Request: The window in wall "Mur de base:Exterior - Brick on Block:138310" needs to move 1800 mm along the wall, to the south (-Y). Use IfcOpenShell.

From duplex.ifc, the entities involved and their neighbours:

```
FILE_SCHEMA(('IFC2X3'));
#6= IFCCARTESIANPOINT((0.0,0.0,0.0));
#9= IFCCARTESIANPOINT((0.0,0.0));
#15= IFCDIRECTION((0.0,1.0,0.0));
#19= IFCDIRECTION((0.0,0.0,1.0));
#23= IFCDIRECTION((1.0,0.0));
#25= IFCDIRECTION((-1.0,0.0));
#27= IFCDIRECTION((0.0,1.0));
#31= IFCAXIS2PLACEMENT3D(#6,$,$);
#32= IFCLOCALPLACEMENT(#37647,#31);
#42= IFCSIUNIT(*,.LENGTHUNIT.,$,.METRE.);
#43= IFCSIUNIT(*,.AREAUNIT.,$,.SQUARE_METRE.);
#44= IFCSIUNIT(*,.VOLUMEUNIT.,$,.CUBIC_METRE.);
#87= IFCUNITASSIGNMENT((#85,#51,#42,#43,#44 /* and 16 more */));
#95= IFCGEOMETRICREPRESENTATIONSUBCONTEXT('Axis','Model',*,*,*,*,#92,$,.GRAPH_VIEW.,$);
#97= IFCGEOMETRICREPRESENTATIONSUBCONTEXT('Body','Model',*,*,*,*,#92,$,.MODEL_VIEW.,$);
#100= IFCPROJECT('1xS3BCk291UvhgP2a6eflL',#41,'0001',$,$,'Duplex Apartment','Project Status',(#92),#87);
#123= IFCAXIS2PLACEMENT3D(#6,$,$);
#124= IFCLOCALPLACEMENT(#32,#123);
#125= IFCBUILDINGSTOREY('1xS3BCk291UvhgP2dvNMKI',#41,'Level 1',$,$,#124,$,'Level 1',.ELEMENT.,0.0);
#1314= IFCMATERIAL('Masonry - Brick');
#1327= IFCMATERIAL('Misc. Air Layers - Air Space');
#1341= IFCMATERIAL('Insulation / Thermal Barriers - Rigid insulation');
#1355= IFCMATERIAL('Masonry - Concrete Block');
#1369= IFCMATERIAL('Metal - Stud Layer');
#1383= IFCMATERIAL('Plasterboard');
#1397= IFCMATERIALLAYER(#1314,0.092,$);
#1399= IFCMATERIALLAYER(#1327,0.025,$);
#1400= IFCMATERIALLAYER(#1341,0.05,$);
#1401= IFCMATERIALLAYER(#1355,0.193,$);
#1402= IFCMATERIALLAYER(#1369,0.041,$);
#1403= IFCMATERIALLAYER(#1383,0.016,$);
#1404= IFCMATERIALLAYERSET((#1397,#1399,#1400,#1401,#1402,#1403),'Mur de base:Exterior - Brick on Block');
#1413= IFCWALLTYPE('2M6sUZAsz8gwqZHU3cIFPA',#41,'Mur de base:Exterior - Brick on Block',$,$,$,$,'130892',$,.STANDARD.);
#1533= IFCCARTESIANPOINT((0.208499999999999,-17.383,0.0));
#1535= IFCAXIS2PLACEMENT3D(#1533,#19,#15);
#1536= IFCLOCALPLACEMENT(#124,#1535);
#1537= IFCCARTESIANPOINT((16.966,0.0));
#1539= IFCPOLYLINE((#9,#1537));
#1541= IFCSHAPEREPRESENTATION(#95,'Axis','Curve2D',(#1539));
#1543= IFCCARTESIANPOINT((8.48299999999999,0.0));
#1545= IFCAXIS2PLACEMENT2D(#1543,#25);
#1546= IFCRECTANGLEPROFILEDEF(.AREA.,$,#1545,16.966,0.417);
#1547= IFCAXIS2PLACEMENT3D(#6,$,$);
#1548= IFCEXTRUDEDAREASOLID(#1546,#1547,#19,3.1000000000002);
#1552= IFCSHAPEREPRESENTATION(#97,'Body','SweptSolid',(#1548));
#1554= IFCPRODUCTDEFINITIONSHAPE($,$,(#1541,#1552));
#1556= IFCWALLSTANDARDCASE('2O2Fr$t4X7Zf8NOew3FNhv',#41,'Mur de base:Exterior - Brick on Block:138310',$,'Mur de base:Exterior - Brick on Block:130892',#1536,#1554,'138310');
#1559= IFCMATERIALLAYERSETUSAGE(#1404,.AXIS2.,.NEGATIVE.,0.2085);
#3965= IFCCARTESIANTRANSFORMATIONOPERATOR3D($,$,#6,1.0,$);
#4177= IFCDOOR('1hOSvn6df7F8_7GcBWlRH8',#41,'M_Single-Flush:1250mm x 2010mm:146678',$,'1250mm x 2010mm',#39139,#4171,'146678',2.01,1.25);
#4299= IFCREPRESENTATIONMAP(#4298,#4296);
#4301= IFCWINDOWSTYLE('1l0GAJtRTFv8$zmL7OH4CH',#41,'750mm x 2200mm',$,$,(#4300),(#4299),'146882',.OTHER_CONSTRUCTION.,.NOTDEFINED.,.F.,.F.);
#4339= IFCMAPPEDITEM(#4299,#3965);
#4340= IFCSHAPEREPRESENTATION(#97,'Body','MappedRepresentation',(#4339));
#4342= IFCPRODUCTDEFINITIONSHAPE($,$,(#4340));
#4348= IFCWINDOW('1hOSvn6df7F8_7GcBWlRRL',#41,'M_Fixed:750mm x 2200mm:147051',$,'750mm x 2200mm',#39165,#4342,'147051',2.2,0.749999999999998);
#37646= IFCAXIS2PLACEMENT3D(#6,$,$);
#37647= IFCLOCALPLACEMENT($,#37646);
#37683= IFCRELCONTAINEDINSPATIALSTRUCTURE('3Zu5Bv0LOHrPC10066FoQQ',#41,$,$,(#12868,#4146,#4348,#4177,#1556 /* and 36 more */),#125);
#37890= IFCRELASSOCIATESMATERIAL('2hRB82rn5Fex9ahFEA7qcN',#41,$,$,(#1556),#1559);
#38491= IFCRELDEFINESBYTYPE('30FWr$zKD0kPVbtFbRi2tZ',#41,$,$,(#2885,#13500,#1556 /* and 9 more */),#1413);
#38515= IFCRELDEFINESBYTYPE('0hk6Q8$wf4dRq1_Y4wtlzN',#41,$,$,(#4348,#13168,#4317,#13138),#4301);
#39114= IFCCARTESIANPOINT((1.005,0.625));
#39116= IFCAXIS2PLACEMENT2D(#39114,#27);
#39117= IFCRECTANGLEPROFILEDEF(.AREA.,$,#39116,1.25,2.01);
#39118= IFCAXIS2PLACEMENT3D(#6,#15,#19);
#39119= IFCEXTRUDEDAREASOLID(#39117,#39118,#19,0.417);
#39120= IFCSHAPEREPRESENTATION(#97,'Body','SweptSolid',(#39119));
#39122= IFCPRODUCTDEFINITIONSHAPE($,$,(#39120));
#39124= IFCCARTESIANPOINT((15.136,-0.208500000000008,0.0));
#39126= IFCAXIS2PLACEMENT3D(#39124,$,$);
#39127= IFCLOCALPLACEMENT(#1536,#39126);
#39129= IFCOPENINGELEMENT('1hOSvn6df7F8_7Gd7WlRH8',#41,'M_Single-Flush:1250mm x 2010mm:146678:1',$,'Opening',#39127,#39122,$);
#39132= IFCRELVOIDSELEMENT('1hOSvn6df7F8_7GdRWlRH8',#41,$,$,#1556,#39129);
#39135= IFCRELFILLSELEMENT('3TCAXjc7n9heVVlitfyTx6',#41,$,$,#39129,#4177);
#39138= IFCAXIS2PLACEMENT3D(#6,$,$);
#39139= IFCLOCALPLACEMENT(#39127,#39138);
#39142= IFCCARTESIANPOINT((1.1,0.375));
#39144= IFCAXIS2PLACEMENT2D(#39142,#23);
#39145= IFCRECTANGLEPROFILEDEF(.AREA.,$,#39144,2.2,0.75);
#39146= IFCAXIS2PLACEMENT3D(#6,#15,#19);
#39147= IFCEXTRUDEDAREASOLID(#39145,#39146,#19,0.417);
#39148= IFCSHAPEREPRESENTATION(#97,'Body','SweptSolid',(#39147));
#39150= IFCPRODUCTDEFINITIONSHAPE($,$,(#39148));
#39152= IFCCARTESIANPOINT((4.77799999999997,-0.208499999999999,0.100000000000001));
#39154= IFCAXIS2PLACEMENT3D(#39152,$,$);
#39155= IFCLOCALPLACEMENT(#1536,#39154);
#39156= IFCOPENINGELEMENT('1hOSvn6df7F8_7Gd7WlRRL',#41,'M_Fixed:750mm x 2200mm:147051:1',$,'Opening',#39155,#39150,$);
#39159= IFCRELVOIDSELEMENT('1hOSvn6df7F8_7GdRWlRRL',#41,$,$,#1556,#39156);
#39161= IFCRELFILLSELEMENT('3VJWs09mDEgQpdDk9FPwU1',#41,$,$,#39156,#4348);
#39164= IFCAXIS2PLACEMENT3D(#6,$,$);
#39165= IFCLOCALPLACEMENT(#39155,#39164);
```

```python
import ifcopenshell
import ifcopenshell.api.geometry
import ifcopenshell.util.placement
import ifcopenshell.util.unit

model = ifcopenshell.open("duplex.ifc")
unit_scale = ifcopenshell.util.unit.calculate_unit_scale(model)

window = model.by_id(4348)
opening = window.FillsVoids[0].RelatingOpeningElement
wall = opening.VoidsElements[0].RelatingBuildingElement

wall_matrix = ifcopenshell.util.placement.get_local_placement(wall.ObjectPlacement)
shift = wall_matrix[:3, 0] * -1.8 / unit_scale
before = ifcopenshell.util.placement.get_local_placement(window.ObjectPlacement)[:3, 3].copy()

# The window is placed relative to its opening, so it follows when the opening moves.
matrix = ifcopenshell.util.placement.get_local_placement(opening.ObjectPlacement)
matrix[:3, 3] += shift
ifcopenshell.api.geometry.edit_object_placement(
    model, product=opening, matrix=matrix, is_si=False, should_transform_children=True
)

after = ifcopenshell.util.placement.get_local_placement(window.ObjectPlacement)[:3, 3]
print("window moved by", (after - before).round(3) + 0.0)

model.write("duplex-out.ifc")
```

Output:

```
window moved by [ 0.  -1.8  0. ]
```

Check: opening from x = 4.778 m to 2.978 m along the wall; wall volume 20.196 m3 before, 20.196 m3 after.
